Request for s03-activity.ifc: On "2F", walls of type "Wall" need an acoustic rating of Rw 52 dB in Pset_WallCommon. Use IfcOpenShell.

First a look at what the model holds.

```python
import ifcopenshell
import ifcopenshell.util.element

model = ifcopenshell.open("s03-activity.ifc")
print(model.schema)
storey = next(s for s in model.by_type("IfcBuildingStorey") if s.Name == "2F")
walls = [e for e in ifcopenshell.util.element.get_decomposition(storey) if e.is_a("IfcWall")]
seen = {}
for e in walls:
    element_type = ifcopenshell.util.element.get_type(e)
    key = (element_type.Name if element_type != e and element_type else None, ifcopenshell.util.element.get_pset(e, "Pset_WallCommon", "AcousticRating"))
    seen[key] = seen.get(key, 0) + 1
for (name, value), count in sorted(seen.items(), key=str):
    print(count, "x", name, "|", value)
```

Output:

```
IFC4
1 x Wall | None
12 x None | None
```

```python
import ifcopenshell
import ifcopenshell.api.pset
import ifcopenshell.util.element

model = ifcopenshell.open("s03-activity.ifc")

storey = next(s for s in model.by_type("IfcBuildingStorey") if s.Name == "2F")
walls = [e for e in ifcopenshell.util.element.get_decomposition(storey) if e.is_a("IfcWall")]

count = 0
for e in walls:
    element_type = ifcopenshell.util.element.get_type(e)
    if element_type in (None, e) or element_type.Name != "Wall":
        continue
    # add_pset returns the element's existing set when there is one.
    pset = ifcopenshell.api.pset.add_pset(model, product=e, name="Pset_WallCommon")
    ifcopenshell.api.pset.edit_pset(model, pset=pset, properties={"AcousticRating": "Rw 52 dB"})
    count += 1

print(count, "walls updated")

model.write("s03-activity_updated.ifc")
```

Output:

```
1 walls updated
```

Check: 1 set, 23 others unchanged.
